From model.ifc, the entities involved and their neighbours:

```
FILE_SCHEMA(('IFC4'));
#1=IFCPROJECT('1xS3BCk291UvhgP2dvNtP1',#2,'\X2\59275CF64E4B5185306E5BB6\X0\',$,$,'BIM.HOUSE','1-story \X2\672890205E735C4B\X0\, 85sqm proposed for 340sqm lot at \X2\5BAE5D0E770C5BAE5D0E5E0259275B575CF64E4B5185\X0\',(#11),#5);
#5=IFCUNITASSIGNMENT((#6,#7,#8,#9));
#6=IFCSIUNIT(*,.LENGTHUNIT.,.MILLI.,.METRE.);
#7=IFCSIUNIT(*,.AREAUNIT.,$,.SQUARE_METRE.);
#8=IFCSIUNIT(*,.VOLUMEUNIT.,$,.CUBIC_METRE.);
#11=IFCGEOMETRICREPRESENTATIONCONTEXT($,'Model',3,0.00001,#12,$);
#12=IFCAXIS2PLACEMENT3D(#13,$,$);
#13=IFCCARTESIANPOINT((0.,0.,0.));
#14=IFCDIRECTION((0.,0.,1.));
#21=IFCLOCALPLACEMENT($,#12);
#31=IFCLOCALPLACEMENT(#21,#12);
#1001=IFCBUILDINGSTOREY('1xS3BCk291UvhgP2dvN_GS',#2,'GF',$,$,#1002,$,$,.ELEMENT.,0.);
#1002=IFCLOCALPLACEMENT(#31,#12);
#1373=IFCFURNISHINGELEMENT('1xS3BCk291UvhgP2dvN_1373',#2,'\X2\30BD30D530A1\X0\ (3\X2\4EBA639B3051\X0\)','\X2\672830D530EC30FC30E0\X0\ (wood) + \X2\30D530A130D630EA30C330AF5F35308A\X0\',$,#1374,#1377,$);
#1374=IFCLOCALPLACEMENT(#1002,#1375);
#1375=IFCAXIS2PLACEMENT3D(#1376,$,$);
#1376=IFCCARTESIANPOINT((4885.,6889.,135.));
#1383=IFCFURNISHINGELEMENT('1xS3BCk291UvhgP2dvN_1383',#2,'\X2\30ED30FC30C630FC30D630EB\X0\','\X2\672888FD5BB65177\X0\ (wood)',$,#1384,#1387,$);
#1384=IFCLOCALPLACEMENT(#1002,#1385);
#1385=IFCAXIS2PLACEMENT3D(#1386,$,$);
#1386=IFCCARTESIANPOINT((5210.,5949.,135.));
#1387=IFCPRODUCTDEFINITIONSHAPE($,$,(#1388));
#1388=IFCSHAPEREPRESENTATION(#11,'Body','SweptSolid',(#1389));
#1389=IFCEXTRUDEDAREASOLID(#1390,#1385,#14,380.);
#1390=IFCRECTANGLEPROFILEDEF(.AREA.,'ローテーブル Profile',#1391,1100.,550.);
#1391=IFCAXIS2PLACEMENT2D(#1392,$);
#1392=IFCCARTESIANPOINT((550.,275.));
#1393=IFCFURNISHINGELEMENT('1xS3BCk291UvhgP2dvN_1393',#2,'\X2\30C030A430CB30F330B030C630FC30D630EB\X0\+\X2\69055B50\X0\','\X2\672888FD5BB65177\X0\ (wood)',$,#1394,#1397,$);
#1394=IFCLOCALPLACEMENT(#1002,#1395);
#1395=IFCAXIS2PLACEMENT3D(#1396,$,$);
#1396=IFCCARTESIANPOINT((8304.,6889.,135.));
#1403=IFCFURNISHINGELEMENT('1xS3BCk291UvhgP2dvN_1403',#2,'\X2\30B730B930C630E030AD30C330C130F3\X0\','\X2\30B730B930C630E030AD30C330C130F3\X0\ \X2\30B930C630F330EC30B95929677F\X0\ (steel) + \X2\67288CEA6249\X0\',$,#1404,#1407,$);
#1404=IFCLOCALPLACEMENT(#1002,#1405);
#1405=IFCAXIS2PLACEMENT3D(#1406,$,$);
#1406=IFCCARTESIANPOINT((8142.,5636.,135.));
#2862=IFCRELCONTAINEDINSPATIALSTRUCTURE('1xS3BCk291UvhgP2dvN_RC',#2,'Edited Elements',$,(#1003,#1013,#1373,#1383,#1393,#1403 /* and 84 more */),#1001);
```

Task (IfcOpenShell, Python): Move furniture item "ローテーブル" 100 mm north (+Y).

```python
import ifcopenshell
import ifcopenshell.api.geometry
import ifcopenshell.util.placement
import ifcopenshell.util.unit

model = ifcopenshell.open("model.ifc")
unit_scale = ifcopenshell.util.unit.calculate_unit_scale(model)

item = model.by_guid("1xS3BCk291UvhgP2dvN_1383")
matrix = ifcopenshell.util.placement.get_local_placement(item.ObjectPlacement)
matrix[1, 3] += 0.1 / unit_scale
ifcopenshell.api.geometry.edit_object_placement(model, product=item, matrix=matrix, is_si=False)

print(ifcopenshell.util.placement.get_local_placement(item.ObjectPlacement).round(3) + 0.0)

model.write("model_updated.ifc")
```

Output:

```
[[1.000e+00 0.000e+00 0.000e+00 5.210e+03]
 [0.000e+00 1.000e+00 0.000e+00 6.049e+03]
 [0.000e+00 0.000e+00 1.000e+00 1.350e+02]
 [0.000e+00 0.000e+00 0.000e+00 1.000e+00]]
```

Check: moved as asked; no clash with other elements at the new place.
